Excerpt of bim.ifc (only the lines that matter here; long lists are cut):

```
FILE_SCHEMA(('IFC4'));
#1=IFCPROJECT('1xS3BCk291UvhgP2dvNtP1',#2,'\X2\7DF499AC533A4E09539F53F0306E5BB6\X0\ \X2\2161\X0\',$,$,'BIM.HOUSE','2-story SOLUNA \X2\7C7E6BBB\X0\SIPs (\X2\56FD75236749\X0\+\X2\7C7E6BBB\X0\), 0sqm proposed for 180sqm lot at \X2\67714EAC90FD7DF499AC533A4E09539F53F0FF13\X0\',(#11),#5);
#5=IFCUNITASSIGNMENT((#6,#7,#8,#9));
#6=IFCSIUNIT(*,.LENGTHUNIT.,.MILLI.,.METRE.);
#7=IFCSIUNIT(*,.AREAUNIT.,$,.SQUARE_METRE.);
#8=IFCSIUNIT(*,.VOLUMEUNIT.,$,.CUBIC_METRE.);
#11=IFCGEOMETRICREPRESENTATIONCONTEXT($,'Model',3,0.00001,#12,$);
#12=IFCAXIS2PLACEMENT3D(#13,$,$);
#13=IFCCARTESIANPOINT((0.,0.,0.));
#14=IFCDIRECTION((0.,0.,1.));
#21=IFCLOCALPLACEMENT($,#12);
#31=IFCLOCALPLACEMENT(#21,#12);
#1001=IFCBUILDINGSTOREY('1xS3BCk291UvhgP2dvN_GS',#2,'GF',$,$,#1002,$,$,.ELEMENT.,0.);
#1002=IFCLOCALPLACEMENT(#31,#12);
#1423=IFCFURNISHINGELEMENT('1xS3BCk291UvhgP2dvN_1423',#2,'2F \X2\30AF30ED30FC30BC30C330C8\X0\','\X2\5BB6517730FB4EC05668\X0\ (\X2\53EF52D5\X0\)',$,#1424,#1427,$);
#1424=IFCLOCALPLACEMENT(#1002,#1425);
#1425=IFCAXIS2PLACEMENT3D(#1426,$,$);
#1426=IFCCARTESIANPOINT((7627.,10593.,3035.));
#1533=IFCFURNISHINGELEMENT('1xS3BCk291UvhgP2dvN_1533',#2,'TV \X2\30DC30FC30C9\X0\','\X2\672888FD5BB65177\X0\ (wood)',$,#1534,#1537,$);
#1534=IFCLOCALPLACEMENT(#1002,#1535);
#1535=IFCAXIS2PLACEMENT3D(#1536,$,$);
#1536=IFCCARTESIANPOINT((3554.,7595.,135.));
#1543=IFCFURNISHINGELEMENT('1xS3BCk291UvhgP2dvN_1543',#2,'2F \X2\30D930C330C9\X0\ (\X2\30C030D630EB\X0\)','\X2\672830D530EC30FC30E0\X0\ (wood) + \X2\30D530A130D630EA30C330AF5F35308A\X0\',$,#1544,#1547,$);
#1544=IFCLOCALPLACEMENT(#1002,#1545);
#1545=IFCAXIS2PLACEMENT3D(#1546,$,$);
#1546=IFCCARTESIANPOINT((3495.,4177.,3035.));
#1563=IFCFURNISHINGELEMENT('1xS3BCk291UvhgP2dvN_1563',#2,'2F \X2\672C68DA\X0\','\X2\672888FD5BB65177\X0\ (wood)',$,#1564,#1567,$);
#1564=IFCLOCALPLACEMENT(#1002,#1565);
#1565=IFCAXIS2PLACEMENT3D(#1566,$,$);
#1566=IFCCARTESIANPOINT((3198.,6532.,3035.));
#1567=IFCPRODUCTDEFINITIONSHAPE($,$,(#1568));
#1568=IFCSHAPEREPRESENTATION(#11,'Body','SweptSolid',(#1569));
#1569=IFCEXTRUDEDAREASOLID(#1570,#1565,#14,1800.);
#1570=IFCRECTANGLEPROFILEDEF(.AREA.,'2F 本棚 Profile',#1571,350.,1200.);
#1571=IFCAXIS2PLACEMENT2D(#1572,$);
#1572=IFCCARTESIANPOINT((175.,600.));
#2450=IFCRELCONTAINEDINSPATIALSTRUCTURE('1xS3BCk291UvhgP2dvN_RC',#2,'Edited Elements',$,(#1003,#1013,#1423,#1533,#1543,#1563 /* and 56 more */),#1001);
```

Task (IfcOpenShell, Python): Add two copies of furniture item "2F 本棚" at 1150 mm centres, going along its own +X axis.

```python
import ifcopenshell
import ifcopenshell.api.geometry
import ifcopenshell.api.root
import ifcopenshell.util.element
import ifcopenshell.util.placement

model = ifcopenshell.open("bim.ifc")


def reuse_history(source, copy):
    """copy_class also copies each property set's owner history, people and application; keep the originals."""
    for rel in copy.IsDefinedBy:
        if rel.is_a("IfcRelDefinesByProperties") and (history := rel.RelatingPropertyDefinition.OwnerHistory):
            rel.RelatingPropertyDefinition.OwnerHistory = source.OwnerHistory
            ifcopenshell.util.element.remove_deep2(model, history)


source = model.by_guid("1xS3BCk291UvhgP2dvN_1563")
base = ifcopenshell.util.placement.get_local_placement(source.ObjectPlacement)
step = base[:3, 0] * 1150.0

for i in range(1, 3):
    copy = ifcopenshell.api.root.copy_class(model, product=source)
    copy.Representation = ifcopenshell.util.element.copy_deep(
        model, source.Representation, exclude=["IfcGeometricRepresentationContext", "IfcRepresentationMap"]
    )
    reuse_history(source, copy)
    matrix = base.copy()
    matrix[:3, 3] += i * step
    print("added at", matrix[:3, 3].round(3) + 0.0)
    ifcopenshell.api.geometry.edit_object_placement(model, product=copy, matrix=matrix, is_si=False)

model.write("bim_edited.ifc")
```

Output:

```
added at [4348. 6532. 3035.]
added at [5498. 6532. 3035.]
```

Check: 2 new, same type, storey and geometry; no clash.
